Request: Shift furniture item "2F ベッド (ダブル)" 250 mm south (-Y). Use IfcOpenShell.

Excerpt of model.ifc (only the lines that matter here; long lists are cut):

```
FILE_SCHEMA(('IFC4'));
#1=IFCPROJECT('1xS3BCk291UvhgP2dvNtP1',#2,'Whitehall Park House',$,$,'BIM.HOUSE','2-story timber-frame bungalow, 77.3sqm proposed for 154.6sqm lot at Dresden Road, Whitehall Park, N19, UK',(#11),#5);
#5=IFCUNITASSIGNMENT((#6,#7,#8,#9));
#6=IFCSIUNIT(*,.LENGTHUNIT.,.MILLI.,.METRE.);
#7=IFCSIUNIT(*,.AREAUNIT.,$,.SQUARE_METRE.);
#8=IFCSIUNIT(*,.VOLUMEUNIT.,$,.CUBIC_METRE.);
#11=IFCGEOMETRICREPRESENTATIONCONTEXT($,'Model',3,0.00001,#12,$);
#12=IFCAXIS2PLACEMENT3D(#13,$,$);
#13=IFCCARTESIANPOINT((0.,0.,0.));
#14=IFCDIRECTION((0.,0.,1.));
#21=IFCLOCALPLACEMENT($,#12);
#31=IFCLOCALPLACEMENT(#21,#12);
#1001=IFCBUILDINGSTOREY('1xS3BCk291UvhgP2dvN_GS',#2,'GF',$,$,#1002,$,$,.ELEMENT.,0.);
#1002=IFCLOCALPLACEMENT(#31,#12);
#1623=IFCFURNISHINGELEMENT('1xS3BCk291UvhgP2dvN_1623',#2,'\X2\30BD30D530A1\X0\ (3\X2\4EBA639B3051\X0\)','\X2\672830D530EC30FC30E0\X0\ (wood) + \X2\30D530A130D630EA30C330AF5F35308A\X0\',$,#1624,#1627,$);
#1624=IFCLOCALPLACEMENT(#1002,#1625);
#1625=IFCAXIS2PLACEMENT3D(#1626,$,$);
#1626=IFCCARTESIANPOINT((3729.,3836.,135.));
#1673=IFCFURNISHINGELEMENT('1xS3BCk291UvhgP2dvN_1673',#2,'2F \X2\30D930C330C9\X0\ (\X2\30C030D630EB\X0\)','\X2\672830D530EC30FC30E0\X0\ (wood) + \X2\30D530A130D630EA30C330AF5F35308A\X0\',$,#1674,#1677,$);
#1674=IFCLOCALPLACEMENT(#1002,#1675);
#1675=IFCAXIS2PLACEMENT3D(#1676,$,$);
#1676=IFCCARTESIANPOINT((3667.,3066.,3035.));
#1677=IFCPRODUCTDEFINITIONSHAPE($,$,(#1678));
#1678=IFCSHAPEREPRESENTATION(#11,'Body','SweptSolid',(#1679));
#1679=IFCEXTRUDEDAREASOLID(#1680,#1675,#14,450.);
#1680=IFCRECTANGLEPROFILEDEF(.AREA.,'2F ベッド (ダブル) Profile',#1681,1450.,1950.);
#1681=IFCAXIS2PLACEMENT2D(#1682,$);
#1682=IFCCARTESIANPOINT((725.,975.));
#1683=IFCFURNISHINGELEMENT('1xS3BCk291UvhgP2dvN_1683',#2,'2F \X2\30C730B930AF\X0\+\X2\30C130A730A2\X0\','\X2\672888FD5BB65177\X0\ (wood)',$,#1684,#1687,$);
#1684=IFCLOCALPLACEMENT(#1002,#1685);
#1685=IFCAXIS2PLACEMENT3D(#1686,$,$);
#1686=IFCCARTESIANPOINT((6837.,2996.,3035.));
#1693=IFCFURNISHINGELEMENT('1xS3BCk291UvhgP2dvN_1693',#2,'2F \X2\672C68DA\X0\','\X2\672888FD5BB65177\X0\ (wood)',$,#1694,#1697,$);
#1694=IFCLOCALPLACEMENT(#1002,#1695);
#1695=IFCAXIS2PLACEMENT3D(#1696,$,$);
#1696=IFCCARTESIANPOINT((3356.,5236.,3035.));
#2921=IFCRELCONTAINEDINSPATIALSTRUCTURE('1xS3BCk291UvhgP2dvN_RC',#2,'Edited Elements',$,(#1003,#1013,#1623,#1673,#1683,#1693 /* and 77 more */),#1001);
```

```python
import ifcopenshell
import ifcopenshell.api.geometry
import ifcopenshell.util.placement

model = ifcopenshell.open("model.ifc")

item = model.by_guid("1xS3BCk291UvhgP2dvN_1673")
matrix = ifcopenshell.util.placement.get_local_placement(item.ObjectPlacement)
matrix[1, 3] -= 250.0
ifcopenshell.api.geometry.edit_object_placement(model, product=item, matrix=matrix, is_si=False)

print(ifcopenshell.util.placement.get_local_placement(item.ObjectPlacement).round(3) + 0.0)

model.write("model_v2.ifc")
```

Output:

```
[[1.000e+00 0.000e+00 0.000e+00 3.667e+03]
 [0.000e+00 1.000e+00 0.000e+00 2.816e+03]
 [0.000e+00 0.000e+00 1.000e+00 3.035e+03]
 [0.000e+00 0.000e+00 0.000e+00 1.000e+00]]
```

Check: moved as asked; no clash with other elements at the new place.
